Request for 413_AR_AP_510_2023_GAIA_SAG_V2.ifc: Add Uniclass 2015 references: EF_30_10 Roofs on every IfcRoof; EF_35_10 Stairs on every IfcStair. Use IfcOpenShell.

First a look at what the model holds.

```python
import ifcopenshell

model = ifcopenshell.open("413_AR_AP_510_2023_GAIA_SAG_V2.ifc")
print(model.schema)
print("classifications:", [c.Name for c in model.by_type("IfcClassification")])
for ifc_class in ("IfcDoor", "IfcRoof", "IfcStair", "IfcWall", "IfcWindow"):
    print(ifc_class, len(model.by_type(ifc_class)))
```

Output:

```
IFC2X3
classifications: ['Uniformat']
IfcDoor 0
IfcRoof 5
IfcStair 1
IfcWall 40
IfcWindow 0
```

```python
import ifcopenshell
import ifcopenshell.api.classification

model = ifcopenshell.open("413_AR_AP_510_2023_GAIA_SAG_V2.ifc")

# IFC2X3 requires Source and Edition and has no link from the project to the system.
system = model.create_entity("IfcClassification", Source="NBS", Edition="2015", Name="Uniclass 2015")

codes = {
    "IfcRoof": ("EF_30_10", "Roofs"),
    "IfcStair": ("EF_35_10", "Stairs"),
}
for ifc_class, (code, name) in codes.items():
    products = model.by_type(ifc_class)
    ifcopenshell.api.classification.add_reference(
        model, products=products, classification=system, identification=code, name=name
    )
    print(code, len(products))

model.write("413_AR_AP_510_2023_GAIA_SAG_V2_v2.ifc")
```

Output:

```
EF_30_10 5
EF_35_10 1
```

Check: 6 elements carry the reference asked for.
